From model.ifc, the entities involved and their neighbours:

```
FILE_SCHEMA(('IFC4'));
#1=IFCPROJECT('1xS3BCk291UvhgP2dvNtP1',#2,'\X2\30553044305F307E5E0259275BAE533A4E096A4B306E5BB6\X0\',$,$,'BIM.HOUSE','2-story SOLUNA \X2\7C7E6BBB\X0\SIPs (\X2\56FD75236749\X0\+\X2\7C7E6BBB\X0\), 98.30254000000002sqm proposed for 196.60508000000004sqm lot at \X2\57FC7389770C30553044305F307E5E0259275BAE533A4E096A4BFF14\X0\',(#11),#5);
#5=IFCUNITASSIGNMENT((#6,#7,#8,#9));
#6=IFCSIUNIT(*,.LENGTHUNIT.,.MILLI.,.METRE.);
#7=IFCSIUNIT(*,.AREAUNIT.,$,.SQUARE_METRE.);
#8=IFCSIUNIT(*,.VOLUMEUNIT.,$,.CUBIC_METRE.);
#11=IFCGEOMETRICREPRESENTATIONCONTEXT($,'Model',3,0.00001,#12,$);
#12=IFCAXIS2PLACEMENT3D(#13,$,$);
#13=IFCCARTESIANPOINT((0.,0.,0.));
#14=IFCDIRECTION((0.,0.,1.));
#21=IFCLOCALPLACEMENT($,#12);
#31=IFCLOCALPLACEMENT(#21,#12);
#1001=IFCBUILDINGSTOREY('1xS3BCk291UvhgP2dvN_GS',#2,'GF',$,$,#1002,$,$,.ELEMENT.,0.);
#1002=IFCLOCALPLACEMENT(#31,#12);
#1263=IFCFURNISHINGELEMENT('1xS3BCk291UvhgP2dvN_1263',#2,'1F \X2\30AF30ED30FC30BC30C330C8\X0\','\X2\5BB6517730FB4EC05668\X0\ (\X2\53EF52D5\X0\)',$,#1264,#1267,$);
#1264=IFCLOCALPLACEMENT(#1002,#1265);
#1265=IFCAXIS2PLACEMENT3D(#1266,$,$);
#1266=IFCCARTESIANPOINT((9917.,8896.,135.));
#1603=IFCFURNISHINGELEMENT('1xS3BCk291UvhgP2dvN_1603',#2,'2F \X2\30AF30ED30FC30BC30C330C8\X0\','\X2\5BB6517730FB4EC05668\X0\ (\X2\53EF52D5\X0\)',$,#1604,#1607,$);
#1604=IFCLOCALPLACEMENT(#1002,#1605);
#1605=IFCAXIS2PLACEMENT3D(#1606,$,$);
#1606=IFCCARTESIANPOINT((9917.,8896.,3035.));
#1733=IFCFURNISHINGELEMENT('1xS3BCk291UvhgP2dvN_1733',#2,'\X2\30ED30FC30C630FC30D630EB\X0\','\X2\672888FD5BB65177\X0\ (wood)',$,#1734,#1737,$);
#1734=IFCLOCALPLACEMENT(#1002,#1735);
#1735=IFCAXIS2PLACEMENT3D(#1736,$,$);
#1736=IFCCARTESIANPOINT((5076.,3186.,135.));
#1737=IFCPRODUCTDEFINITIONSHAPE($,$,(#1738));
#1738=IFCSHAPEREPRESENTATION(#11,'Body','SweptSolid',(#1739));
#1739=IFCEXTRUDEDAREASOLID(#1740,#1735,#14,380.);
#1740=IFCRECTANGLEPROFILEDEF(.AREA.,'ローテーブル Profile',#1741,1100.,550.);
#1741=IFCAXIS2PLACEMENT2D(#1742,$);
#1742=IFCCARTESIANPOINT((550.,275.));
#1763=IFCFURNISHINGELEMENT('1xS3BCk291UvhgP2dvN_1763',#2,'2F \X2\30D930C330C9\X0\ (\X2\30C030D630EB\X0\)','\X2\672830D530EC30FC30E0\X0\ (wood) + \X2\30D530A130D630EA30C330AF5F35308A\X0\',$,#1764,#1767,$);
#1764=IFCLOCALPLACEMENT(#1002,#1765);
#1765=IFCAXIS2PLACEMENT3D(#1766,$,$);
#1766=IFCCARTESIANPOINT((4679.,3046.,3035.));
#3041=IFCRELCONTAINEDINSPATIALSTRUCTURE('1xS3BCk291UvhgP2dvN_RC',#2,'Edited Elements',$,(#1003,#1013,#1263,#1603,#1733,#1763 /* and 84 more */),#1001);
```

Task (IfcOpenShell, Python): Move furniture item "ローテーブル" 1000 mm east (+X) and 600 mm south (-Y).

```python
import ifcopenshell
import ifcopenshell.api.geometry
import ifcopenshell.util.placement
import ifcopenshell.util.unit

model = ifcopenshell.open("model.ifc")
unit_scale = ifcopenshell.util.unit.calculate_unit_scale(model)

item = model.by_id(1733)
matrix = ifcopenshell.util.placement.get_local_placement(item.ObjectPlacement)
matrix[0, 3] += 1 / unit_scale
matrix[1, 3] -= 0.6 / unit_scale
ifcopenshell.api.geometry.edit_object_placement(model, product=item, matrix=matrix, is_si=False)

print(ifcopenshell.util.placement.get_local_placement(item.ObjectPlacement).round(3) + 0.0)

model.write("model-out.ifc")
```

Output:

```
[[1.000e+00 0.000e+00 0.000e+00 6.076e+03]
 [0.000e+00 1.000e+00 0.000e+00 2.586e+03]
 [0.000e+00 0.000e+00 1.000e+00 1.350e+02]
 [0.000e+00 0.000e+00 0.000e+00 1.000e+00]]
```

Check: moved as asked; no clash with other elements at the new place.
